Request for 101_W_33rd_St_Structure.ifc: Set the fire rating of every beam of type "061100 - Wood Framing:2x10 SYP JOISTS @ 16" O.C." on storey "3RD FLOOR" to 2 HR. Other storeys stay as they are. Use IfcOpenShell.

First a look at what the model holds.

```python
import ifcopenshell
import ifcopenshell.util.element

model = ifcopenshell.open("101_W_33rd_St_Structure.ifc")
print(model.schema)
storey = next(s for s in model.by_type("IfcBuildingStorey") if s.Name == "3RD FLOOR")
beams = [e for e in ifcopenshell.util.element.get_decomposition(storey) if e.is_a("IfcBeam")]
seen = {}
for e in beams:
    element_type = ifcopenshell.util.element.get_type(e)
    key = (element_type.Name if element_type != e and element_type else None, ifcopenshell.util.element.get_pset(e, "Pset_BeamCommon", "FireRating"))
    seen[key] = seen.get(key, 0) + 1
for (name, value), count in sorted(seen.items(), key=str):
    print(count, "x", name, "|", value)
```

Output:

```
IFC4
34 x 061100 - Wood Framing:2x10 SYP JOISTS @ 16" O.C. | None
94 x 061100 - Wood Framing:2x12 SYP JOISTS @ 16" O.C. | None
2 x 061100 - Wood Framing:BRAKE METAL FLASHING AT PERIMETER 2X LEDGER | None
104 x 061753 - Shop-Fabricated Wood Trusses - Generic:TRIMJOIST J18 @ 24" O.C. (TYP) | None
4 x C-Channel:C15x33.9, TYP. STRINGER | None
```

```python
import ifcopenshell
import ifcopenshell.api.pset
import ifcopenshell.util.element

model = ifcopenshell.open("101_W_33rd_St_Structure.ifc")

storey = next(s for s in model.by_type("IfcBuildingStorey") if s.Name == "3RD FLOOR")
beams = [e for e in ifcopenshell.util.element.get_decomposition(storey) if e.is_a("IfcBeam")]

count = 0
for e in beams:
    element_type = ifcopenshell.util.element.get_type(e)
    if element_type in (None, e) or element_type.Name != '061100 - Wood Framing:2x10 SYP JOISTS @ 16" O.C.':
        continue
    # add_pset returns the element's existing set when there is one.
    pset = ifcopenshell.api.pset.add_pset(model, product=e, name="Pset_BeamCommon")
    ifcopenshell.api.pset.edit_pset(model, pset=pset, properties={"FireRating": "2 HR"})
    count += 1

print(count, "beams updated")

model.write("101_W_33rd_St_Structure_edited.ifc")
```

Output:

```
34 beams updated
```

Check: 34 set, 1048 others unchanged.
